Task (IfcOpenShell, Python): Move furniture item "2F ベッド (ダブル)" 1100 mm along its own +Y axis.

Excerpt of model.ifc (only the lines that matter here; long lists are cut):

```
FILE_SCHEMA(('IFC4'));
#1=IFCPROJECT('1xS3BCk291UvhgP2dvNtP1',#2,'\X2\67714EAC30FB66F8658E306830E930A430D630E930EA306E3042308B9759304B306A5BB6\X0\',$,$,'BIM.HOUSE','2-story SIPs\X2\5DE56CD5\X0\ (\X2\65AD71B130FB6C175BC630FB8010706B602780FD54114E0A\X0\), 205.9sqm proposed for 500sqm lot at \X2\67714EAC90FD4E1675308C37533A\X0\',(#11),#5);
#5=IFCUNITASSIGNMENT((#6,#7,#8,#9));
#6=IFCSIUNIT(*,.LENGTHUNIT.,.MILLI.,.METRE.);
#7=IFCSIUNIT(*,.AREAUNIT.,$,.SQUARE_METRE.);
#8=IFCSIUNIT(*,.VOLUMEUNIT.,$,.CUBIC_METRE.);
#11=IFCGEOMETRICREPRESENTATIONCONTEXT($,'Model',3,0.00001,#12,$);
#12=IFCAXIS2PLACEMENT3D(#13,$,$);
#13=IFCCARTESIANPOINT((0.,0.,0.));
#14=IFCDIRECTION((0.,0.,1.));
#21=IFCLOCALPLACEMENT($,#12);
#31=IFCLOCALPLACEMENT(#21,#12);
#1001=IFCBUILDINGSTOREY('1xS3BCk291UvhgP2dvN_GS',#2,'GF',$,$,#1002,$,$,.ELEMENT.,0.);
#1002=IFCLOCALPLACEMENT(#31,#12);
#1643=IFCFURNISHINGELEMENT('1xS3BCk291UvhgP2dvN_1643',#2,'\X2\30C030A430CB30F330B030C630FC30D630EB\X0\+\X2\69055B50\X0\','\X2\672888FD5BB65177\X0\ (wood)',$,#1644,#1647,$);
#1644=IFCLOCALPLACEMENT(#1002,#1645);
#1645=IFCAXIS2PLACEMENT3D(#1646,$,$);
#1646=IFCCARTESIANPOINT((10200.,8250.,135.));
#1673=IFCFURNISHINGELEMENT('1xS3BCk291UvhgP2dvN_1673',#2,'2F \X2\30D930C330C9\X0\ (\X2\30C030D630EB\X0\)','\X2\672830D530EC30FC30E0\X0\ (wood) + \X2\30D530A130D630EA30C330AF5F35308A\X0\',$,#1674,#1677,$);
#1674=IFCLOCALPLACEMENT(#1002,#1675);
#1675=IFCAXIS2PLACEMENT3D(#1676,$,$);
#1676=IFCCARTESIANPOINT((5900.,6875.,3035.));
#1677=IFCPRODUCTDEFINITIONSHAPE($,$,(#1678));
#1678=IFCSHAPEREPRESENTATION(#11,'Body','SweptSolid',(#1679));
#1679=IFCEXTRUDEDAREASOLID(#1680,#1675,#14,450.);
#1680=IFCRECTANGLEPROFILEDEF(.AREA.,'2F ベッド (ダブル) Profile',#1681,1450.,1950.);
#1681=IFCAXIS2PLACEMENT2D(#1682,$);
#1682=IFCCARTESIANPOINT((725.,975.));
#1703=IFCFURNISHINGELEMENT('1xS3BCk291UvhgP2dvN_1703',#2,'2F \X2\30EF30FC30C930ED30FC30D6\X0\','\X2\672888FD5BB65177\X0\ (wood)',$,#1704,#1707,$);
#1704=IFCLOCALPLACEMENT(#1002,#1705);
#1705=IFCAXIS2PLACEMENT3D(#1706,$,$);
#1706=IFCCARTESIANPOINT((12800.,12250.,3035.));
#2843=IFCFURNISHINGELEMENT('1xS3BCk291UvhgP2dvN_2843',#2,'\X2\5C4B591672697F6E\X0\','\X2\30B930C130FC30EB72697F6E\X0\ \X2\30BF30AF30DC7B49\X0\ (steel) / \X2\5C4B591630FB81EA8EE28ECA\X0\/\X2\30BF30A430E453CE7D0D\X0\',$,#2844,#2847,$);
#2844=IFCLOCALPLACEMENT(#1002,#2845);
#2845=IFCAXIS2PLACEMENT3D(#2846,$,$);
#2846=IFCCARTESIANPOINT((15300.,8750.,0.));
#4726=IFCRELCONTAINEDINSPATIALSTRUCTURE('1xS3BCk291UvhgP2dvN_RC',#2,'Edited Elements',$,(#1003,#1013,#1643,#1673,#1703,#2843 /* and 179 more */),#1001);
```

```python
import ifcopenshell
import ifcopenshell.api.geometry
import ifcopenshell.util.placement
import ifcopenshell.util.unit

model = ifcopenshell.open("model.ifc")
unit_scale = ifcopenshell.util.unit.calculate_unit_scale(model)

item = model.by_guid("1xS3BCk291UvhgP2dvN_1673")
matrix = ifcopenshell.util.placement.get_local_placement(item.ObjectPlacement)
matrix[:3, 3] += matrix[:3, 1] * 1.1 / unit_scale
ifcopenshell.api.geometry.edit_object_placement(model, product=item, matrix=matrix, is_si=False)

print(ifcopenshell.util.placement.get_local_placement(item.ObjectPlacement).round(3) + 0.0)

model.write("model-out.ifc")
```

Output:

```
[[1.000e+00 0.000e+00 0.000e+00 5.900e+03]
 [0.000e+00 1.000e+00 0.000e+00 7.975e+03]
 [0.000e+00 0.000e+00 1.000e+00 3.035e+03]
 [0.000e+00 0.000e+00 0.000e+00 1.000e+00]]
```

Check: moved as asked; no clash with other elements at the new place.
